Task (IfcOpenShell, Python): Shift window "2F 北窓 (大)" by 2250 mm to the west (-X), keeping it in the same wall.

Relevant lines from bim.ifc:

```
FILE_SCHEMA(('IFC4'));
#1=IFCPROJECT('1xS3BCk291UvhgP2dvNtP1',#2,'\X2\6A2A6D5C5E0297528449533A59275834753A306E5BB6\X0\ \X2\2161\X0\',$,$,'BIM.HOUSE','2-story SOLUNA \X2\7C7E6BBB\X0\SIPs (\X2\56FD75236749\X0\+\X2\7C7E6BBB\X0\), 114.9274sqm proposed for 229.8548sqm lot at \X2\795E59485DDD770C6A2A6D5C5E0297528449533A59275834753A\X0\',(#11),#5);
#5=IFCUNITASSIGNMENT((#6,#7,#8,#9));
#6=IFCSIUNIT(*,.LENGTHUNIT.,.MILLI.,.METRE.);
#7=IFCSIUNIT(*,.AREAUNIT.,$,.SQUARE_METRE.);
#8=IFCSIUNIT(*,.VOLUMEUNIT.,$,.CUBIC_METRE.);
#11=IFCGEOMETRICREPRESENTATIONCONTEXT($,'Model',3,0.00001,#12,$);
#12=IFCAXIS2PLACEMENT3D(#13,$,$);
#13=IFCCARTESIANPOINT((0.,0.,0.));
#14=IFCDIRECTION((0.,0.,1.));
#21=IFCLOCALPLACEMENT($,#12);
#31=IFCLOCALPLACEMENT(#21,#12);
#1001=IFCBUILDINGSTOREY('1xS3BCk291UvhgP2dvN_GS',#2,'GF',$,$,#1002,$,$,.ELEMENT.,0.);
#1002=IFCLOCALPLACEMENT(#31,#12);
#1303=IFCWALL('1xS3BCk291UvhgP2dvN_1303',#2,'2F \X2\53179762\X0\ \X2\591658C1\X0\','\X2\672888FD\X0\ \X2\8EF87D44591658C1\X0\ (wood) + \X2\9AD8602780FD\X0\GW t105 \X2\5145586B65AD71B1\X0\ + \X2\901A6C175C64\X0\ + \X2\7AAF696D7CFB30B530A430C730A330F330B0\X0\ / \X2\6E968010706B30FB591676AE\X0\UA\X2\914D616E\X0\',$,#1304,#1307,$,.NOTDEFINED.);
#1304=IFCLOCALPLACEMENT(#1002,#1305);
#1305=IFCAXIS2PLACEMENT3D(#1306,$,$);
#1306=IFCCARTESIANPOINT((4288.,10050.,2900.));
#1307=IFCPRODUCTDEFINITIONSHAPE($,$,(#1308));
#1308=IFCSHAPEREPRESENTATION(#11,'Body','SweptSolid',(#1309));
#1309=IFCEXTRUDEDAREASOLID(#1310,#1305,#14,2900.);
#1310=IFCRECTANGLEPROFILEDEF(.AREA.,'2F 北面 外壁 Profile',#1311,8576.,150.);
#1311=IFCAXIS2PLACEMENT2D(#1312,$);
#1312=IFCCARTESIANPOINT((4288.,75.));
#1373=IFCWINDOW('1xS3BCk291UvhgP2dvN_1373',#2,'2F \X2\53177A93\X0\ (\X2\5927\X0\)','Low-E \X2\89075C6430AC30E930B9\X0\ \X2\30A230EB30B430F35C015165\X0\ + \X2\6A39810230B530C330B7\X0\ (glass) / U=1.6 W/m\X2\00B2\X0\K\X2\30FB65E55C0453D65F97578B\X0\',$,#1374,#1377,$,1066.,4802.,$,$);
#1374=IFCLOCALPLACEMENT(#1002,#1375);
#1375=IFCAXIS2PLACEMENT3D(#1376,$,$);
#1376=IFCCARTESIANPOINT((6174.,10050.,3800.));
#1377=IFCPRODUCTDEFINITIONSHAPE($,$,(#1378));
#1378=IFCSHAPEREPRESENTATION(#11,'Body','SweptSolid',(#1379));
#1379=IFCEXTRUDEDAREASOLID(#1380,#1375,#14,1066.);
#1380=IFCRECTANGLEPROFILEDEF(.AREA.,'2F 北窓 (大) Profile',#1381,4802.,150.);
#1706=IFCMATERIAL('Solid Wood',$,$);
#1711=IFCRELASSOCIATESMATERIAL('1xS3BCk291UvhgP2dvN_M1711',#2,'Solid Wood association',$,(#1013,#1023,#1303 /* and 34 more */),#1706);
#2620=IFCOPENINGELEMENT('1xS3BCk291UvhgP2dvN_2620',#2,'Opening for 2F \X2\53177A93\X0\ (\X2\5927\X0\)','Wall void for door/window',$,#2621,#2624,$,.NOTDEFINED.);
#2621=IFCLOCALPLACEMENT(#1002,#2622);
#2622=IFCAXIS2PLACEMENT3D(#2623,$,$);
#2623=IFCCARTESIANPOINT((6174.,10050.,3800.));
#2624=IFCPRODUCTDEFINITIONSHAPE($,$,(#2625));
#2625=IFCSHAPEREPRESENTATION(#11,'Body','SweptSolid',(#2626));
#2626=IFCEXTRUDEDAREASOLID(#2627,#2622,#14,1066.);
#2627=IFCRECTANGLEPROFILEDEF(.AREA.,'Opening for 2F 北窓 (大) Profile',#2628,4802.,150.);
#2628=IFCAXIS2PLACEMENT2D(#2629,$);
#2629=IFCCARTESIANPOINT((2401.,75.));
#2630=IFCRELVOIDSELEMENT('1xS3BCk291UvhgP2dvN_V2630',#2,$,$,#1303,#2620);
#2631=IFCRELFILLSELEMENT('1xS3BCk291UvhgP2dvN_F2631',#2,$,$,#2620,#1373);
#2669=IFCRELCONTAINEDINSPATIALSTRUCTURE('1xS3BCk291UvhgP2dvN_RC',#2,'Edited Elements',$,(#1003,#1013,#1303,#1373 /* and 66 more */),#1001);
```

```python
import ifcopenshell
import ifcopenshell.api.geometry
import ifcopenshell.util.placement

model = ifcopenshell.open("bim.ifc")

window = model.by_guid("1xS3BCk291UvhgP2dvN_1373")
opening = window.FillsVoids[0].RelatingOpeningElement
wall = opening.VoidsElements[0].RelatingBuildingElement

wall_matrix = ifcopenshell.util.placement.get_local_placement(wall.ObjectPlacement)
shift = wall_matrix[:3, 0] * -2250.0
before = ifcopenshell.util.placement.get_local_placement(window.ObjectPlacement)[:3, 3].copy()

# The window is not placed relative to its opening, so move both.
for product in (opening, window):
    matrix = ifcopenshell.util.placement.get_local_placement(product.ObjectPlacement)
    matrix[:3, 3] += shift
    ifcopenshell.api.geometry.edit_object_placement(model, product=product, matrix=matrix, is_si=False)

after = ifcopenshell.util.placement.get_local_placement(window.ObjectPlacement)[:3, 3]
print("window moved by", (after - before).round(3) + 0.0)

model.write("bim_updated.ifc")
```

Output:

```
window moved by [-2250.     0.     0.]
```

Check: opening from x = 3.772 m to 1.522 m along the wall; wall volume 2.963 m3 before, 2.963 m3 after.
